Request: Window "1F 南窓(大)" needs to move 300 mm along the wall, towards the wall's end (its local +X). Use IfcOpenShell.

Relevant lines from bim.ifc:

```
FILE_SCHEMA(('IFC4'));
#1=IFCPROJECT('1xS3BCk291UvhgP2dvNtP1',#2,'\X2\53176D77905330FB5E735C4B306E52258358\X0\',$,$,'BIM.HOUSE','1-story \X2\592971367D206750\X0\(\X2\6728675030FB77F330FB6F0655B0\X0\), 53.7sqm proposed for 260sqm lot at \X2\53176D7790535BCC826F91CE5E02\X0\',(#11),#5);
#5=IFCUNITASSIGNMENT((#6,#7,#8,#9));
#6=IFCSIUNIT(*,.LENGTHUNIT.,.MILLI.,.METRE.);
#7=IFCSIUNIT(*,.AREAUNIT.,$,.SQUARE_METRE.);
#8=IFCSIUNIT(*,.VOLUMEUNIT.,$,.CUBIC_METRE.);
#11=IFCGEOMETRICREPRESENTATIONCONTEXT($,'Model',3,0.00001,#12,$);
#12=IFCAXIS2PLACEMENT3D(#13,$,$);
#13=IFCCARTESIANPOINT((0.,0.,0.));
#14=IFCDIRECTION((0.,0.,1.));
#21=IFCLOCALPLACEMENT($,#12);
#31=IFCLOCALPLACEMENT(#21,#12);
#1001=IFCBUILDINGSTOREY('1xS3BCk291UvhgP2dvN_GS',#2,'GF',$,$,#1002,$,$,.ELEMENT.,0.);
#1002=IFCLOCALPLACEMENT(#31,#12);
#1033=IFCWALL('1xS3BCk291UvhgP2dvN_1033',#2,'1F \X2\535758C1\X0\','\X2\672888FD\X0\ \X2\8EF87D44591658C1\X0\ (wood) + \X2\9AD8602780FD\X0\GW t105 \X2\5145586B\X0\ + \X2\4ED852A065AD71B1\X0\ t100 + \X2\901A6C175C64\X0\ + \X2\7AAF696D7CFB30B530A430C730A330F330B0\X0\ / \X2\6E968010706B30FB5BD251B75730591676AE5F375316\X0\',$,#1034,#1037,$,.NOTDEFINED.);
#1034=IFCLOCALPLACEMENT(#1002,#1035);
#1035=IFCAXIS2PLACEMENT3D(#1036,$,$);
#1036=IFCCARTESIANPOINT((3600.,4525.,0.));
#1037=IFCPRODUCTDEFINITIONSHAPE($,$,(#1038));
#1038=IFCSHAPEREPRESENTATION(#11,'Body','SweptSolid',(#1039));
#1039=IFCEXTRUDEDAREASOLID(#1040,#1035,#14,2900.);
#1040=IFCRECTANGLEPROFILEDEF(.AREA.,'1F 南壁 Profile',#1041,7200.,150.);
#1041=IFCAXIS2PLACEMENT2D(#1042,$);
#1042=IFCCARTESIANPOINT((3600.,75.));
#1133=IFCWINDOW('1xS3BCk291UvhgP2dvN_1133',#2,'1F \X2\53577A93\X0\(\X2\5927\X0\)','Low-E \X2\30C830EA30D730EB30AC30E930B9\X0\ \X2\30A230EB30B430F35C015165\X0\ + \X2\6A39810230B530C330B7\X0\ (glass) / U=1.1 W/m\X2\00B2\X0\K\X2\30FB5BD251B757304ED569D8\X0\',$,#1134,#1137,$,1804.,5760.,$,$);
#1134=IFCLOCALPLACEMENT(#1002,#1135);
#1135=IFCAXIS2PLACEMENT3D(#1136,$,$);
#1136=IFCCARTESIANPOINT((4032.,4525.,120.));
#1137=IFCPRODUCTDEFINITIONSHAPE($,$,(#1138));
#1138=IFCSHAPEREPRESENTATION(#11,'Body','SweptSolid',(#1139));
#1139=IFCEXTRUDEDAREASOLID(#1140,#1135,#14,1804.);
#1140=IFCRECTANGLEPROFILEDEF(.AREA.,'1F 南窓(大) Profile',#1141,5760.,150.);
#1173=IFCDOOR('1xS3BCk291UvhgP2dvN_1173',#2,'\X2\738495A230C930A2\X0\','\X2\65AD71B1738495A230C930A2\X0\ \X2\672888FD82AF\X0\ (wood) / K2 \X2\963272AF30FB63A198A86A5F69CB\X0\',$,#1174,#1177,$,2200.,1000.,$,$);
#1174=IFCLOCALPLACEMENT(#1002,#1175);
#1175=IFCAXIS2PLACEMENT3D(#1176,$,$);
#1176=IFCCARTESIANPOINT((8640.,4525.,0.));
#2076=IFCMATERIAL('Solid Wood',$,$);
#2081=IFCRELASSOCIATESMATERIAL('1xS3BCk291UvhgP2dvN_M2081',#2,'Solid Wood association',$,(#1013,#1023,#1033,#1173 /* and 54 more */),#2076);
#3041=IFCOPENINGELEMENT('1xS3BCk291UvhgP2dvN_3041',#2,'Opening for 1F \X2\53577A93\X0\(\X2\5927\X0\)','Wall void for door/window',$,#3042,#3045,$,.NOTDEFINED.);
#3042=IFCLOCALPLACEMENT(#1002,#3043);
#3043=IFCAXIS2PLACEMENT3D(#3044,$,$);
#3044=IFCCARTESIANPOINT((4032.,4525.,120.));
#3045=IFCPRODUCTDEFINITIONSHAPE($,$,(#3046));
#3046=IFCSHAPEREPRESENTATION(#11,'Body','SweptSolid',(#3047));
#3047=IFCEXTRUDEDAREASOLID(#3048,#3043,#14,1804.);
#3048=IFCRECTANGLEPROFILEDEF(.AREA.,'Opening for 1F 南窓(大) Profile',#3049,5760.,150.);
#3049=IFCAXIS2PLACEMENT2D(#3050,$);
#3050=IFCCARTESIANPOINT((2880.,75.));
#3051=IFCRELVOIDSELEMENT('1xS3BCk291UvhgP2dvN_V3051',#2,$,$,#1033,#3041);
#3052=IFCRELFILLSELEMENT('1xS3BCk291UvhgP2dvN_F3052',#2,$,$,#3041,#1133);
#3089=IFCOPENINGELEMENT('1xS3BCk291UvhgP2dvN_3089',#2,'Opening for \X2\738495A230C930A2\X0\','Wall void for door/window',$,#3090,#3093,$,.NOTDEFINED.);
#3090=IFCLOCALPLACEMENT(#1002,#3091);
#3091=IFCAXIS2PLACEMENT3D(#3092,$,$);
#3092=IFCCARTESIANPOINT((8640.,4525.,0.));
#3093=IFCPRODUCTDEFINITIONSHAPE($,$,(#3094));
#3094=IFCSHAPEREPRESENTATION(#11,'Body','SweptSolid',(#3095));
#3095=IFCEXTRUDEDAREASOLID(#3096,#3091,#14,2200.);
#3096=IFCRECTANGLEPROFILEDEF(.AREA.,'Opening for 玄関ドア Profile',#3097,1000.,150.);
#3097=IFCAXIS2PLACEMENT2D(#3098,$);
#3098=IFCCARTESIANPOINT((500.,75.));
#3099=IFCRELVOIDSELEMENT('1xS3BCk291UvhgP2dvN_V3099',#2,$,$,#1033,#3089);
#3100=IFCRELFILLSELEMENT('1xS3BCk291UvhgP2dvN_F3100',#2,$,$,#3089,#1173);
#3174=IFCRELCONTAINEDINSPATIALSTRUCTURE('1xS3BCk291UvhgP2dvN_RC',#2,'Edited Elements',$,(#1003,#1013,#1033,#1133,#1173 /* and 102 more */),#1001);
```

```python
import ifcopenshell
import ifcopenshell.api.geometry
import ifcopenshell.util.placement
import ifcopenshell.util.unit

model = ifcopenshell.open("bim.ifc")
unit_scale = ifcopenshell.util.unit.calculate_unit_scale(model)

window = model.by_guid("1xS3BCk291UvhgP2dvN_1133")
opening = window.FillsVoids[0].RelatingOpeningElement
wall = opening.VoidsElements[0].RelatingBuildingElement

wall_matrix = ifcopenshell.util.placement.get_local_placement(wall.ObjectPlacement)
shift = wall_matrix[:3, 0] * 0.3 / unit_scale
before = ifcopenshell.util.placement.get_local_placement(window.ObjectPlacement)[:3, 3].copy()

# The window is not placed relative to its opening, so move both.
for product in (opening, window):
    matrix = ifcopenshell.util.placement.get_local_placement(product.ObjectPlacement)
    matrix[:3, 3] += shift
    ifcopenshell.api.geometry.edit_object_placement(model, product=product, matrix=matrix, is_si=False)

after = ifcopenshell.util.placement.get_local_placement(window.ObjectPlacement)[:3, 3]
print("window moved by", (after - before).round(3) + 0.0)

model.write("bim-out.ifc")
```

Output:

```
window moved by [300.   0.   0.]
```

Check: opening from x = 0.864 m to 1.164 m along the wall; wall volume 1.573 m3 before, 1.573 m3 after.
